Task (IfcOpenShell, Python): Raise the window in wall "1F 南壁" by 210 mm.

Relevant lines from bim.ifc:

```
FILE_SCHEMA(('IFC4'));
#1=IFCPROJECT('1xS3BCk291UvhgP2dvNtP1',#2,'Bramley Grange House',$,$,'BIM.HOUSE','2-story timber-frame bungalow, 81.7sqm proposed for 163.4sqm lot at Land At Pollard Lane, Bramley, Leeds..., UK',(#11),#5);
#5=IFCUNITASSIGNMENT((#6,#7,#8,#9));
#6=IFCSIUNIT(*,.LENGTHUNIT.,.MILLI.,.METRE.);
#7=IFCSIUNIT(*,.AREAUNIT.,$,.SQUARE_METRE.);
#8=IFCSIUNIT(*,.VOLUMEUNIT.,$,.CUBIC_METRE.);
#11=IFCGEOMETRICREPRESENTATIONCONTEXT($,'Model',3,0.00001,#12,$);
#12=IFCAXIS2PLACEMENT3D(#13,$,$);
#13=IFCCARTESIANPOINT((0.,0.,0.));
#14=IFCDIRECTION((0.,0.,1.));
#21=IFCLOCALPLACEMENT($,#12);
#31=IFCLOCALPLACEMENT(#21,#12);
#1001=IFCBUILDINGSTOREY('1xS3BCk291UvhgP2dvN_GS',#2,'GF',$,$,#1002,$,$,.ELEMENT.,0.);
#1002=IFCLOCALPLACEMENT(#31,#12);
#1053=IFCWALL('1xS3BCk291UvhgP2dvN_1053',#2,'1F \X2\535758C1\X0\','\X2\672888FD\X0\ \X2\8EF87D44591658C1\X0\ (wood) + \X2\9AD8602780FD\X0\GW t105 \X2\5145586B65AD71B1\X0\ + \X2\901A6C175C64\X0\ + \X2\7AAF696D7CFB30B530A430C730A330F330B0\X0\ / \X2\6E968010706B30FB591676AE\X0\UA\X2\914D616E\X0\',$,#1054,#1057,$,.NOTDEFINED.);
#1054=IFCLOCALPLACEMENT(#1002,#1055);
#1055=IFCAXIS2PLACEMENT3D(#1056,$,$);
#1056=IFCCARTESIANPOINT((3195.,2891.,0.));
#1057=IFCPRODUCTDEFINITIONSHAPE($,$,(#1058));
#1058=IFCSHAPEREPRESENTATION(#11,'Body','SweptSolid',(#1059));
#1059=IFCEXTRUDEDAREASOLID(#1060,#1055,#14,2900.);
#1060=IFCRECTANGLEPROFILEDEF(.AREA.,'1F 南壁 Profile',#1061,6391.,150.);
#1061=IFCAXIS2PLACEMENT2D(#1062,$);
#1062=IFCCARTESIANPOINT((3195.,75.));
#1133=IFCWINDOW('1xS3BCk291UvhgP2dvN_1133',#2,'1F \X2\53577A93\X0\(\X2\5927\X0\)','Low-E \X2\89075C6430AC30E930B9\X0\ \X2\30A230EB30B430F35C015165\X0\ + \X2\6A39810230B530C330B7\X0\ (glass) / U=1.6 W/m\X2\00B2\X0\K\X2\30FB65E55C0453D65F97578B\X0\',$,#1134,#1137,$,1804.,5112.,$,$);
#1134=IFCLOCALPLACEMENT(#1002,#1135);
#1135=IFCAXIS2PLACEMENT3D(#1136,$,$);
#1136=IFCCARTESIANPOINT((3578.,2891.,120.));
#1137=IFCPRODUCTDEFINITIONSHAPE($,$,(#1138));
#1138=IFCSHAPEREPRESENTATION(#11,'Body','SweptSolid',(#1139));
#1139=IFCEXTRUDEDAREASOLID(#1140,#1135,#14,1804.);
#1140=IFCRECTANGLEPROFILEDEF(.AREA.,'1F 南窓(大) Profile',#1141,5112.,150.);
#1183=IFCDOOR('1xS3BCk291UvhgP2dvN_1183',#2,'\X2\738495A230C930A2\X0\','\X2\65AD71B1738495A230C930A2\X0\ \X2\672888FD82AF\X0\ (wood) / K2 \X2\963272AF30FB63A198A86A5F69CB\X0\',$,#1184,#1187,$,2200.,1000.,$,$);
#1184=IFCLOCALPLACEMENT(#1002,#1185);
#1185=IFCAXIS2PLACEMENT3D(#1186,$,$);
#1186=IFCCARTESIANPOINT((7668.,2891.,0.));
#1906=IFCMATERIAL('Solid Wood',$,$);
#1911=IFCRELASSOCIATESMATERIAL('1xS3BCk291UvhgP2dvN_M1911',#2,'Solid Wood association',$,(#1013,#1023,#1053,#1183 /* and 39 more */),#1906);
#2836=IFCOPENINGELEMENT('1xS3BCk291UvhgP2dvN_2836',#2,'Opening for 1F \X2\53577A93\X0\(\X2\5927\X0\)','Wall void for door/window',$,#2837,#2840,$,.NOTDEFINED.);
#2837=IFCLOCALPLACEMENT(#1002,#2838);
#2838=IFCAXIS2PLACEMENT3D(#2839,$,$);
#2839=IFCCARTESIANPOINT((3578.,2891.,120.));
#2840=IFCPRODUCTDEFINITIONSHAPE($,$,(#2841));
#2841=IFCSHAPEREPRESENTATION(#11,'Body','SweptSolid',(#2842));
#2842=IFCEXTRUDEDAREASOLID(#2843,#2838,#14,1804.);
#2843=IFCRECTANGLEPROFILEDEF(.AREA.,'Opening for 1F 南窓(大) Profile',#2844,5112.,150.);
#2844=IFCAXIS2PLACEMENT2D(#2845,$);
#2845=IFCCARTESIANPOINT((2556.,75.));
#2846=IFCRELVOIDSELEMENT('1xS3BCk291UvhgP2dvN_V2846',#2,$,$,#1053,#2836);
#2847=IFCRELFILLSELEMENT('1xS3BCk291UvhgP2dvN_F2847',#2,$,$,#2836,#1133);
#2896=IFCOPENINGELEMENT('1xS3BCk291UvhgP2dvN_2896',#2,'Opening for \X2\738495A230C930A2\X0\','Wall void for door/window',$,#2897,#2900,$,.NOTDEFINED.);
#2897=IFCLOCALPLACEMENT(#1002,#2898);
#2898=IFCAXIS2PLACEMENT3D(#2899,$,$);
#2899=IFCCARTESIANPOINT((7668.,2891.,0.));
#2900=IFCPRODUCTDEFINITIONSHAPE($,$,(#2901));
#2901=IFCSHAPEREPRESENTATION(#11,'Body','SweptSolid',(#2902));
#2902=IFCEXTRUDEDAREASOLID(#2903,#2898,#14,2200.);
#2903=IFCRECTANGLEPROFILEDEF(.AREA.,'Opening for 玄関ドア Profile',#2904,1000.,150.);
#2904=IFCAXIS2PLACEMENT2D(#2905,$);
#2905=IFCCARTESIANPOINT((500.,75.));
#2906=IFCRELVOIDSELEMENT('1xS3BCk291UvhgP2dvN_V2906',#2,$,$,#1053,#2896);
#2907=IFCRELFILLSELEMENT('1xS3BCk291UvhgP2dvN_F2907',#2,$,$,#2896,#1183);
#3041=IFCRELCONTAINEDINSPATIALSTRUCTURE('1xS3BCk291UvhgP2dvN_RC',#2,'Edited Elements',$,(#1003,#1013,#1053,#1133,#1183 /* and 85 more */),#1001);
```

```python
import numpy as np
import ifcopenshell
import ifcopenshell.api.geometry
import ifcopenshell.util.placement
import ifcopenshell.util.unit

model = ifcopenshell.open("bim.ifc")
unit_scale = ifcopenshell.util.unit.calculate_unit_scale(model)

window = model.by_guid("1xS3BCk291UvhgP2dvN_1133")
opening = window.FillsVoids[0].RelatingOpeningElement
dz = 210.0

shift = np.array([0.0, 0.0, dz])
# The window is not placed relative to its opening, so move both.
for product in (opening, window):
    matrix = ifcopenshell.util.placement.get_local_placement(product.ObjectPlacement)
    matrix[:3, 3] += shift
    ifcopenshell.api.geometry.edit_object_placement(model, product=product, matrix=matrix, is_si=False)

print(f"moved by {dz * unit_scale:+.3f} m")

model.write("bim_updated.ifc")
```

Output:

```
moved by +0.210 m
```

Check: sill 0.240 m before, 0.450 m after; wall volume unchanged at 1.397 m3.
